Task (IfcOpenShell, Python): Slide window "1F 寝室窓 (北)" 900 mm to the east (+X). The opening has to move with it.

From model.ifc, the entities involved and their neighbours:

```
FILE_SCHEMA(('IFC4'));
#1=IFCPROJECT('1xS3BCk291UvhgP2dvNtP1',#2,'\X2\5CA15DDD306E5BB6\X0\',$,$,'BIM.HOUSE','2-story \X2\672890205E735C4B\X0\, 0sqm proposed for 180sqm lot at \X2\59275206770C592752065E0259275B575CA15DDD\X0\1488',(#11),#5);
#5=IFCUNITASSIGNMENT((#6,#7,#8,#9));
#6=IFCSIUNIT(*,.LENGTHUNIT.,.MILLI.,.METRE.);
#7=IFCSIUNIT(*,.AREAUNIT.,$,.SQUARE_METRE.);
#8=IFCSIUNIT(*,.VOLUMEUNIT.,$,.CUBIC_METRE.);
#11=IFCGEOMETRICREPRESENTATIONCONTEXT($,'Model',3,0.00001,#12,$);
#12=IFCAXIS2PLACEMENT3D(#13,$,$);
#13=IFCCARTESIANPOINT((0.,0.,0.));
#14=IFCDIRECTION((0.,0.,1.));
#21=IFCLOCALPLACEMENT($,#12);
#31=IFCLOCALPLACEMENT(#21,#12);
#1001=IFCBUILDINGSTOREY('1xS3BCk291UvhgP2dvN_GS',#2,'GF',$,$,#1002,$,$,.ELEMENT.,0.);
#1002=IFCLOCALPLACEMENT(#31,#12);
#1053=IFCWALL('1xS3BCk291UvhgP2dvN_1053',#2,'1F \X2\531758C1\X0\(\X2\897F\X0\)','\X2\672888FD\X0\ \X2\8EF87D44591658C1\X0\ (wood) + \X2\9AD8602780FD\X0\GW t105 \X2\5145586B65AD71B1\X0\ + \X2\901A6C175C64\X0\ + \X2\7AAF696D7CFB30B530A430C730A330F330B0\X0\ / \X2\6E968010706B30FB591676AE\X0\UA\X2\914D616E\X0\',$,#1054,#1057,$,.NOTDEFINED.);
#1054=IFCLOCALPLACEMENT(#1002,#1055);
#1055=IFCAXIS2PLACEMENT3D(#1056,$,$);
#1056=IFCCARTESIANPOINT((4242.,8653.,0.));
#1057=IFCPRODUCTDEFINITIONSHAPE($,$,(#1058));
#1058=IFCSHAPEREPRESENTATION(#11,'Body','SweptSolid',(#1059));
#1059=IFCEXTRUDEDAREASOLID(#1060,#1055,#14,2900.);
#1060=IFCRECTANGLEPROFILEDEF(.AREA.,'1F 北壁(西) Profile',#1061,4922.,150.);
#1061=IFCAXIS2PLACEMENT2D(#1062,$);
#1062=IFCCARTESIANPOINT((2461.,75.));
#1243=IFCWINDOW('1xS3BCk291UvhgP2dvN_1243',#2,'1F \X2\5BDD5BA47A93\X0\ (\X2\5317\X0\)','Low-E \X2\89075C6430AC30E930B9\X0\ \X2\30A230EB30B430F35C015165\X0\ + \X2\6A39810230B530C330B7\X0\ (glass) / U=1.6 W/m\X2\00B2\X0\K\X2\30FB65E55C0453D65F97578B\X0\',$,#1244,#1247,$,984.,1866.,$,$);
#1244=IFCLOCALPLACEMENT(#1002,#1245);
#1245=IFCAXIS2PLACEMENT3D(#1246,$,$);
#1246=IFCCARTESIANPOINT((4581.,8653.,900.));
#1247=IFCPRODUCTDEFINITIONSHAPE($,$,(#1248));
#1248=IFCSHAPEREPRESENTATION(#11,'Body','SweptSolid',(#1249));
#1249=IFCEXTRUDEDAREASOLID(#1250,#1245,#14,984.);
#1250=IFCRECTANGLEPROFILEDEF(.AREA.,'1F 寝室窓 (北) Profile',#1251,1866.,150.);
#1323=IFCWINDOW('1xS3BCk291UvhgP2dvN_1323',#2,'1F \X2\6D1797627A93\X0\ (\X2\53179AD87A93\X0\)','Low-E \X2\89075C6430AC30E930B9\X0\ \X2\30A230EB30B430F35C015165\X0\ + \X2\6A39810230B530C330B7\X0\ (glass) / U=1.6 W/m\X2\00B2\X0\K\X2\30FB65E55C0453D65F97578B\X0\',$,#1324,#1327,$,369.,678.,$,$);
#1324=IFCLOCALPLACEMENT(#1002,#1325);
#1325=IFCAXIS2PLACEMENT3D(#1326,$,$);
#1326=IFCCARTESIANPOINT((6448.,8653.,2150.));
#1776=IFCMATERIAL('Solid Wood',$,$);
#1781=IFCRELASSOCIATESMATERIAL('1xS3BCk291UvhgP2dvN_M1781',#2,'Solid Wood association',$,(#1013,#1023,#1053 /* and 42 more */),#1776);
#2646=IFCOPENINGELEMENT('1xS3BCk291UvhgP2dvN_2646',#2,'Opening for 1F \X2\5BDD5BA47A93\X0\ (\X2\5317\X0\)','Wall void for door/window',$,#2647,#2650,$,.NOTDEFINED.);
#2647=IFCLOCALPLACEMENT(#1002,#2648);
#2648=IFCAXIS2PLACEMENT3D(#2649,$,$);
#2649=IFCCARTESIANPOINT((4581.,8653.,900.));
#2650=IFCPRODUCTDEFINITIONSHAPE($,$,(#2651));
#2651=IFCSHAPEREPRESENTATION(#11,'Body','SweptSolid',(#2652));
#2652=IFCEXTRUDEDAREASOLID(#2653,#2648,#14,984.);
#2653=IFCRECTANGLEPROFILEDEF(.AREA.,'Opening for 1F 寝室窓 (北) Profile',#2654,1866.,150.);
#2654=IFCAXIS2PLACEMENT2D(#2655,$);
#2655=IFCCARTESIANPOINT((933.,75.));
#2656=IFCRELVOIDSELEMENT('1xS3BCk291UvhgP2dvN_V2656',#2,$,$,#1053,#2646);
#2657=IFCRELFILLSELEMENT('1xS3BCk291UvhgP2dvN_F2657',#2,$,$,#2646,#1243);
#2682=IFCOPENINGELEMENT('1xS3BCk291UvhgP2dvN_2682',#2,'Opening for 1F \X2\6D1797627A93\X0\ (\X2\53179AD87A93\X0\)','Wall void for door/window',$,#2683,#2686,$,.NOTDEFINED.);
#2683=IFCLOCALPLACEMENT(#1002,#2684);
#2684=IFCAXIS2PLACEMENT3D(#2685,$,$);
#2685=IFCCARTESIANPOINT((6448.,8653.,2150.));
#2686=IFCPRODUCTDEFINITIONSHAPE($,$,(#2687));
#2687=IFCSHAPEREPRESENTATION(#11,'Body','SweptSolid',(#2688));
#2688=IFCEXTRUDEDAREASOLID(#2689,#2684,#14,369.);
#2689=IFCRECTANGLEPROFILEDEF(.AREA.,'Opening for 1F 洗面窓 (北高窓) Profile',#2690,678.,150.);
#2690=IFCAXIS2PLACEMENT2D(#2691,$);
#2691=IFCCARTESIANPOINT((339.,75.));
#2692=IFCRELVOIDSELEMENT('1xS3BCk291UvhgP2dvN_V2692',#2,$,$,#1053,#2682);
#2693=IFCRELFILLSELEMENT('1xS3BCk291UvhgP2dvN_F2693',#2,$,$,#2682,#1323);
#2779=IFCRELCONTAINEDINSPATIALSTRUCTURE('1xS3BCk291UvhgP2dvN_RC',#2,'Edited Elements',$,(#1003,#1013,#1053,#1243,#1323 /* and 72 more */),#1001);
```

```python
import ifcopenshell
import ifcopenshell.api.geometry
import ifcopenshell.util.placement
import ifcopenshell.util.unit

model = ifcopenshell.open("model.ifc")
unit_scale = ifcopenshell.util.unit.calculate_unit_scale(model)

window = model.by_id(1243)
opening = window.FillsVoids[0].RelatingOpeningElement
wall = opening.VoidsElements[0].RelatingBuildingElement

wall_matrix = ifcopenshell.util.placement.get_local_placement(wall.ObjectPlacement)
shift = wall_matrix[:3, 0] * 0.9 / unit_scale
before = ifcopenshell.util.placement.get_local_placement(window.ObjectPlacement)[:3, 3].copy()

# The window is not placed relative to its opening, so move both.
for product in (opening, window):
    matrix = ifcopenshell.util.placement.get_local_placement(product.ObjectPlacement)
    matrix[:3, 3] += shift
    ifcopenshell.api.geometry.edit_object_placement(model, product=product, matrix=matrix, is_si=False)

after = ifcopenshell.util.placement.get_local_placement(window.ObjectPlacement)[:3, 3]
print("window moved by", (after - before).round(3) + 0.0)

model.write("model-out.ifc")
```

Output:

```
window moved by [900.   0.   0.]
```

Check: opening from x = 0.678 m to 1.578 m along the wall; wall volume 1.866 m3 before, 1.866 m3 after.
